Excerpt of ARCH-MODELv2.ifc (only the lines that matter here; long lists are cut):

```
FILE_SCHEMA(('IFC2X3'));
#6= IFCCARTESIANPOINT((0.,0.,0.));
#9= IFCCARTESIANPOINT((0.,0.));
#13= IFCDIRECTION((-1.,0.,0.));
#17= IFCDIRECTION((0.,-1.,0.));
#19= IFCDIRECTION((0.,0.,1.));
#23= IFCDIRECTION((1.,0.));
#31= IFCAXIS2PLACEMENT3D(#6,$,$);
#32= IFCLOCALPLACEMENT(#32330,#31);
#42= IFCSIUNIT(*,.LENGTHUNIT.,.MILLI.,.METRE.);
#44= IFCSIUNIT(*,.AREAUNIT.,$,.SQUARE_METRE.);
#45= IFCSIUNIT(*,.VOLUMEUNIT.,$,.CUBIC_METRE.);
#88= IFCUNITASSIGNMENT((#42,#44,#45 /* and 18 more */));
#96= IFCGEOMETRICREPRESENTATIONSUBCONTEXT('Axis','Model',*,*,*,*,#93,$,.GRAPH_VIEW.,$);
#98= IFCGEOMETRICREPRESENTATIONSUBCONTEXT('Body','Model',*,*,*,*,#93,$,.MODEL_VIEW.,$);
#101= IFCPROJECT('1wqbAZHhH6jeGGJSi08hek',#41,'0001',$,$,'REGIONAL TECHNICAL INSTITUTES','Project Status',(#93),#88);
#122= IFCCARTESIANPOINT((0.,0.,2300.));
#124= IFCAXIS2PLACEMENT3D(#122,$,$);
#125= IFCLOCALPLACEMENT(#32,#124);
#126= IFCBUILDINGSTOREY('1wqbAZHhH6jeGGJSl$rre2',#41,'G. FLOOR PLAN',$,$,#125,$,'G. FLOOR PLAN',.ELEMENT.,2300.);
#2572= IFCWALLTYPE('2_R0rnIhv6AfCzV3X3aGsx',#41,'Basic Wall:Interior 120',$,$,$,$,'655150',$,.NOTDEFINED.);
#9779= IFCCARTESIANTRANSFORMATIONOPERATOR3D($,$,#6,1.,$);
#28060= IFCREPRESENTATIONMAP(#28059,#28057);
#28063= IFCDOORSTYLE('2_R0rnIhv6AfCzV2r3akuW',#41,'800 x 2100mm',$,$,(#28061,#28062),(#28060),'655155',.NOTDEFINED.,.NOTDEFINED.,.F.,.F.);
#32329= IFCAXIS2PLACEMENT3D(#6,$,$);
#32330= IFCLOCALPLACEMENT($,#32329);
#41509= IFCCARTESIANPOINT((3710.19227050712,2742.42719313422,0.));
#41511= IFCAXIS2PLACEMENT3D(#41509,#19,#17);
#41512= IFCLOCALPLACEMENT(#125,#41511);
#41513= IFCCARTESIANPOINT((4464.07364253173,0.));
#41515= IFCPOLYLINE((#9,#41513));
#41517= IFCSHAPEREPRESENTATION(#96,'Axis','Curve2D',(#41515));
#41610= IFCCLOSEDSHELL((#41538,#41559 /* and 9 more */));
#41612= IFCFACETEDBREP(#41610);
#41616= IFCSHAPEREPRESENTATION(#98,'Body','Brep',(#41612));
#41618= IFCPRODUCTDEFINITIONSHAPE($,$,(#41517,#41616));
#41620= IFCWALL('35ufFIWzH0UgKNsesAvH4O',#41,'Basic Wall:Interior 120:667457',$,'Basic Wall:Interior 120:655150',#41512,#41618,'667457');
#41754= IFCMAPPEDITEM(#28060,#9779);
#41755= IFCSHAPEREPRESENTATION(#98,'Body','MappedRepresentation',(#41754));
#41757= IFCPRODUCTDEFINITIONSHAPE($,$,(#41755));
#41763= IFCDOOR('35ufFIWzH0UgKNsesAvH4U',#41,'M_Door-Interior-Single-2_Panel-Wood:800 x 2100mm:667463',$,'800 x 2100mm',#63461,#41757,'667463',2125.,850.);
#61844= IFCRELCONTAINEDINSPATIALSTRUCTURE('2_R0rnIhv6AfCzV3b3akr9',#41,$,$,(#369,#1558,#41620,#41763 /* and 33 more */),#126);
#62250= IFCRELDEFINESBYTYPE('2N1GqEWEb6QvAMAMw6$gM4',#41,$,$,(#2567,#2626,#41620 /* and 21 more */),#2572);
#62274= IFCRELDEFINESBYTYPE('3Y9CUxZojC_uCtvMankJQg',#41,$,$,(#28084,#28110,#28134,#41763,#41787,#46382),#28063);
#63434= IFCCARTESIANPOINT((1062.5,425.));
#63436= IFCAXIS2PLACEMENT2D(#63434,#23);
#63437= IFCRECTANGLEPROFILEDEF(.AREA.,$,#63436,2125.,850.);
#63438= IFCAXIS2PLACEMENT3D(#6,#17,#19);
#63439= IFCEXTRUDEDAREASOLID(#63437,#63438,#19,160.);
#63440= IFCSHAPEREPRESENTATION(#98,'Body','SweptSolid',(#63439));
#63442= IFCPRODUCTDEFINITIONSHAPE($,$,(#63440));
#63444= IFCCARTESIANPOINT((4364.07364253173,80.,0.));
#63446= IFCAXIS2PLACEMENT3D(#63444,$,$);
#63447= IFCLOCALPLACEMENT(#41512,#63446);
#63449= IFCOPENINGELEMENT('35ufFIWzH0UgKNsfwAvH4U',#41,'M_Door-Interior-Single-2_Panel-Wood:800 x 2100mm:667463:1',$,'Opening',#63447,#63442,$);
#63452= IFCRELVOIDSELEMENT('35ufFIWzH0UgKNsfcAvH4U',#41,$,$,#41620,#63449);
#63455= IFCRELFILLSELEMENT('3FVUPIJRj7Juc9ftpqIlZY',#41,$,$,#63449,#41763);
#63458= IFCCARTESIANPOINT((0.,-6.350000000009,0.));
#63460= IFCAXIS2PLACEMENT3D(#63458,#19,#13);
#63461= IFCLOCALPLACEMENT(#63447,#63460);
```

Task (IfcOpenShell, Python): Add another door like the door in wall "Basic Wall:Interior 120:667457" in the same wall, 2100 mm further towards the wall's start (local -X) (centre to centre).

```python
import ifcopenshell
import ifcopenshell.api.feature
import ifcopenshell.api.geometry
import ifcopenshell.api.root
import ifcopenshell.geom
import ifcopenshell.util.element
import ifcopenshell.util.placement
import ifcopenshell.util.shape

model = ifcopenshell.open("ARCH-MODELv2.ifc")
settings = ifcopenshell.geom.settings()


def volume(element):
    """Net volume in cubic metres, openings subtracted."""
    shape = ifcopenshell.geom.create_shape(settings, element)
    return ifcopenshell.util.shape.get_volume(shape.geometry)


def reuse_history(source, copy):
    """copy_class also copies each property set's owner history, people and application; keep the originals."""
    for rel in copy.IsDefinedBy:
        if rel.is_a("IfcRelDefinesByProperties") and (history := rel.RelatingPropertyDefinition.OwnerHistory):
            rel.RelatingPropertyDefinition.OwnerHistory = source.OwnerHistory
            ifcopenshell.util.element.remove_deep2(model, history)


door = model.by_guid("35ufFIWzH0UgKNsesAvH4U")
opening = door.FillsVoids[0].RelatingOpeningElement
wall = opening.VoidsElements[0].RelatingBuildingElement
before = volume(wall)
shift = ifcopenshell.util.placement.get_local_placement(wall.ObjectPlacement)[:3, 0] * -2100.0

# copy_class copies the void relationship, type, container and properties, but no geometry.
new_opening = ifcopenshell.api.root.copy_class(model, product=opening)
new_opening.Representation = ifcopenshell.util.element.copy_deep(
    model, opening.Representation, exclude=["IfcGeometricRepresentationContext", "IfcRepresentationMap"]
)
new_opening.Name = "M_Door-Interior-Single-2_Panel-Wood:800 x 2100mm"
new_door = ifcopenshell.api.root.copy_class(model, product=door)
new_door.Representation = ifcopenshell.util.element.copy_deep(
    model, door.Representation, exclude=["IfcGeometricRepresentationContext", "IfcRepresentationMap"]
)
new_door.Name = "M_Door-Interior-Single-2_Panel-Wood:800 x 2100mm"
new_door.Tag = None
reuse_history(door, new_door)
fills = ifcopenshell.api.feature.add_filling(model, opening=new_opening, element=new_door)
fills.OwnerHistory = new_door.OwnerHistory  # required in IFC2X3

for old, new in ((opening, new_opening), (door, new_door)):
    matrix = ifcopenshell.util.placement.get_local_placement(old.ObjectPlacement)
    matrix[:3, 3] += shift
    ifcopenshell.api.geometry.edit_object_placement(model, product=new, matrix=matrix, is_si=False)

after = volume(wall)

print(f"wall volume {before:.3f} -> {after:.3f} m3")

model.write("ARCH-MODELv2_edited.ifc")
```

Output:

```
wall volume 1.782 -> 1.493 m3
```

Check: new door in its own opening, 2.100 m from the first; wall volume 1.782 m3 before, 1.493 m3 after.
